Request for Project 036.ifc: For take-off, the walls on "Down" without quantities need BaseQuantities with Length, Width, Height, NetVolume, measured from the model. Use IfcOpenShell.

First a look at what the model holds.

```python
import ifcopenshell
import ifcopenshell.util.element
import ifcopenshell.util.unit

model = ifcopenshell.open("Project 036.ifc")
print(model.schema)
for unit_type in ("LENGTHUNIT", "AREAUNIT", "VOLUMEUNIT"):
    print(unit_type, ifcopenshell.util.unit.calculate_unit_scale(model, unit_type))
storey = next(s for s in model.by_type("IfcBuildingStorey") if s.Name == "Down")
walls = [e for e in ifcopenshell.util.element.get_decomposition(storey) if e.is_a("IfcWall")]
for e in sorted(walls, key=lambda e: e.id()):
    print(e.id(), e.is_a(), e.Name, list(ifcopenshell.util.element.get_psets(e, qtos_only=True)), sep=" | ")
```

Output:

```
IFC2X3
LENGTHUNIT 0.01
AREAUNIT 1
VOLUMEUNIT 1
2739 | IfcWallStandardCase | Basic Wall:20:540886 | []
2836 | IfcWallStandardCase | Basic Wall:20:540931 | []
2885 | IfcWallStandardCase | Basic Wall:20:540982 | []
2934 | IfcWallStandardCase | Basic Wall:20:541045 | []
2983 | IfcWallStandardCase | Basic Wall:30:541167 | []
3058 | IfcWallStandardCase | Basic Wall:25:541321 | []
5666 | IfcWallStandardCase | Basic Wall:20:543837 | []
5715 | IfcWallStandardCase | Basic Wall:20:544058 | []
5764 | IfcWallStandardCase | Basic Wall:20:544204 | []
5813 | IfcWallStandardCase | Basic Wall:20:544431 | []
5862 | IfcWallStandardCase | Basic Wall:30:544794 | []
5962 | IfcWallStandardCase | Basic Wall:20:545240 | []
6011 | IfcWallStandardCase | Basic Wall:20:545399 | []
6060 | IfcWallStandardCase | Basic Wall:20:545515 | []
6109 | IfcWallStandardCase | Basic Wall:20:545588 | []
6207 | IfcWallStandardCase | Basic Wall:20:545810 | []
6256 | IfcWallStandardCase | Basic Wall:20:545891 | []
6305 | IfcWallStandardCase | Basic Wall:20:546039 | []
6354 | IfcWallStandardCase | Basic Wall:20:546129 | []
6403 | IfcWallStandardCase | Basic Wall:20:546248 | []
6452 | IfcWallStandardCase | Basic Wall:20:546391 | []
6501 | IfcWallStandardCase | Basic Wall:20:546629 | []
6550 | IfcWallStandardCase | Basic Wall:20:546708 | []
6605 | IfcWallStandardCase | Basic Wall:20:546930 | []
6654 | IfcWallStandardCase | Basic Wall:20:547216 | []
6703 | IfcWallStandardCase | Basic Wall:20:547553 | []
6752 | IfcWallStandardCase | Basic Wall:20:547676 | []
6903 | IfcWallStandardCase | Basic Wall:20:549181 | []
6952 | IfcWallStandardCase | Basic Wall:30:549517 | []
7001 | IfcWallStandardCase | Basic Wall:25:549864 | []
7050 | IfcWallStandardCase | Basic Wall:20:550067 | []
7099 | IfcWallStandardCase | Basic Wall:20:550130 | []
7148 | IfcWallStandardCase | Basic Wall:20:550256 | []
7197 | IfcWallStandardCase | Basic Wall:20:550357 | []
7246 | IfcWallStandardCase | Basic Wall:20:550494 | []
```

```python
import ifcopenshell
import ifcopenshell.api.pset
import ifcopenshell.geom
import ifcopenshell.util.element
import ifcopenshell.util.shape
import ifcopenshell.util.unit

model = ifcopenshell.open("Project 036.ifc")
unit_scale = ifcopenshell.util.unit.calculate_unit_scale(model)
volume_scale = ifcopenshell.util.unit.calculate_unit_scale(model, "VOLUMEUNIT")
settings = ifcopenshell.geom.settings()

storey = next(s for s in model.by_type("IfcBuildingStorey") if s.Name == "Down")
walls = [e for e in ifcopenshell.util.element.get_decomposition(storey) if e.is_a("IfcWall")]

for e in sorted(walls, key=lambda e: e.id()):
    if ifcopenshell.util.element.get_psets(e, qtos_only=True, should_inherit=False):
        continue
    # Geometry comes back in metres, in the element's own axes.
    shape = ifcopenshell.geom.create_shape(settings, e)
    values = {
        "Length": ifcopenshell.util.shape.get_x(shape.geometry) / unit_scale,
        "Width": ifcopenshell.util.shape.get_y(shape.geometry) / unit_scale,
        "Height": ifcopenshell.util.shape.get_z(shape.geometry) / unit_scale,
        "NetVolume": ifcopenshell.util.shape.get_volume(shape.geometry) / volume_scale,
    }
    qto = ifcopenshell.api.pset.add_qto(model, product=e, name="BaseQuantities")
    ifcopenshell.api.pset.edit_qto(model, qto=qto, properties=values)
    print(e.id(), {k: round(v, 3) for k, v in values.items()})

model.write("Project 036-out.ifc")
```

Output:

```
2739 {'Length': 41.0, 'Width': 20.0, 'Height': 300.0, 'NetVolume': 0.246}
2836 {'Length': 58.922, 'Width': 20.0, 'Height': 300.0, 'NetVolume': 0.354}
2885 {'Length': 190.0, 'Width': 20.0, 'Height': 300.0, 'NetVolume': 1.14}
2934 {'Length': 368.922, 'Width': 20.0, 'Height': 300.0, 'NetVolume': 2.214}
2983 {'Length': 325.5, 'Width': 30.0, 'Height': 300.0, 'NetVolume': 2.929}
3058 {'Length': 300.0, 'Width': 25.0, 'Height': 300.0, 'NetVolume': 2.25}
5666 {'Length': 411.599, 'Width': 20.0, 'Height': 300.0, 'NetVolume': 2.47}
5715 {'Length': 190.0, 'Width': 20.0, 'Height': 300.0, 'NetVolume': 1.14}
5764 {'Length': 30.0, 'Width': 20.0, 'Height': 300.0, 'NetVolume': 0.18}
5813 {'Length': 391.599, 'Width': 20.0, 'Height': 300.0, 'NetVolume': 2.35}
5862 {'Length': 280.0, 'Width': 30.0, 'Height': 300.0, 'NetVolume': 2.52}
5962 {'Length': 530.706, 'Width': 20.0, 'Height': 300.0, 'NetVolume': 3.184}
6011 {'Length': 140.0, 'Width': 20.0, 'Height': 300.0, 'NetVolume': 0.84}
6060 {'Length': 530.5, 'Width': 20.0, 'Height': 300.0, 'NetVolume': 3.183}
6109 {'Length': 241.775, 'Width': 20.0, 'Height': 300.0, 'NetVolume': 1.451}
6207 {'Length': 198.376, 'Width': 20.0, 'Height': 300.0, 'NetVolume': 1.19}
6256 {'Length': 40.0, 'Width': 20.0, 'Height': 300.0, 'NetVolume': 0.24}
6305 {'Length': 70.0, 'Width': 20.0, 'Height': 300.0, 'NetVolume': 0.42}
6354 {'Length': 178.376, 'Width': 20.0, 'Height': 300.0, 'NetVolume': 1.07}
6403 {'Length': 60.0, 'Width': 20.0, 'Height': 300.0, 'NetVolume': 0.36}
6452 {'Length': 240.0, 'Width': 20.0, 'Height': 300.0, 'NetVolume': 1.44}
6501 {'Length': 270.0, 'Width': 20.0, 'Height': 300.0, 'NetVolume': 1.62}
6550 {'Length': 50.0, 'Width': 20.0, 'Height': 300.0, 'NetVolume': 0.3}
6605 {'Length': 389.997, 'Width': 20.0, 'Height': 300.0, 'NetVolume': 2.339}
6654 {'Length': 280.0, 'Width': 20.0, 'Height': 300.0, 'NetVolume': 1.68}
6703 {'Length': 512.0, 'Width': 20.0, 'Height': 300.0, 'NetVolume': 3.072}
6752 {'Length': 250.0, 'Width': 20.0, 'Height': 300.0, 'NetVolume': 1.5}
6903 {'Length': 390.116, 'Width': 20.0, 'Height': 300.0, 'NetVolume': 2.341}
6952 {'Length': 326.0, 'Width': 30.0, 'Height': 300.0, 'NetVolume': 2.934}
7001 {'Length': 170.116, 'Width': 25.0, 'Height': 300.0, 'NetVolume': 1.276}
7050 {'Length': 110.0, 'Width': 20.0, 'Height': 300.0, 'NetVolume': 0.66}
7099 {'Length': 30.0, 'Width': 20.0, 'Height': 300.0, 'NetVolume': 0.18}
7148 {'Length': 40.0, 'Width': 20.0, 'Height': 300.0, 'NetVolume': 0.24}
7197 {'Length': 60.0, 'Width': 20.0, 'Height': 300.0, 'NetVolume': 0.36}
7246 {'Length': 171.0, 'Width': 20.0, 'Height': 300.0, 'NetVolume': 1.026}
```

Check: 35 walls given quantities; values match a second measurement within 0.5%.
